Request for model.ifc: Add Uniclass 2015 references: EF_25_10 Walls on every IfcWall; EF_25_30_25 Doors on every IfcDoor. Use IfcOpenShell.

First a look at what the model holds.

```python
import ifcopenshell

model = ifcopenshell.open("model.ifc")
print(model.schema)
print("classifications:", [c.Name for c in model.by_type("IfcClassification")])
for ifc_class in ("IfcDoor", "IfcRoof", "IfcStair", "IfcWall", "IfcWindow"):
    print(ifc_class, len(model.by_type(ifc_class)))
```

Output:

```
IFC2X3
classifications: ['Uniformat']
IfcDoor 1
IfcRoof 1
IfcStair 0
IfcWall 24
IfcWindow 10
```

```python
import ifcopenshell
import ifcopenshell.api.classification

model = ifcopenshell.open("model.ifc")

# IFC2X3 requires Source and Edition and has no link from the project to the system.
system = model.create_entity("IfcClassification", Source="NBS", Edition="2015", Name="Uniclass 2015")

codes = {
    "IfcWall": ("EF_25_10", "Walls"),
    "IfcDoor": ("EF_25_30_25", "Doors"),
}
for ifc_class, (code, name) in codes.items():
    products = model.by_type(ifc_class)
    ifcopenshell.api.classification.add_reference(
        model, products=products, classification=system, identification=code, name=name
    )
    print(code, len(products))

model.write("model_rev.ifc")
```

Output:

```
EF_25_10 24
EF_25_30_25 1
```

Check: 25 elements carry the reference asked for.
